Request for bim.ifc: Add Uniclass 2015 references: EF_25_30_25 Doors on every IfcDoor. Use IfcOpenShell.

First a look at what the model holds.

```python
import ifcopenshell

model = ifcopenshell.open("bim.ifc")
print(model.schema)
print("classifications:", [c.Name for c in model.by_type("IfcClassification")])
for ifc_class in ("IfcDoor", "IfcRoof", "IfcStair", "IfcWall", "IfcWindow"):
    print(ifc_class, len(model.by_type(ifc_class)))
```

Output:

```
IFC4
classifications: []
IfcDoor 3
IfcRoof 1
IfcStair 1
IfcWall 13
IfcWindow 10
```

```python
import ifcopenshell
import ifcopenshell.api.classification

model = ifcopenshell.open("bim.ifc")

system = ifcopenshell.api.classification.add_classification(model, classification="Uniclass 2015")

codes = {
    "IfcDoor": ("EF_25_30_25", "Doors"),
}
for ifc_class, (code, name) in codes.items():
    products = model.by_type(ifc_class)
    ifcopenshell.api.classification.add_reference(
        model, products=products, classification=system, identification=code, name=name
    )
    print(code, len(products))

model.write("bim_rev.ifc")
```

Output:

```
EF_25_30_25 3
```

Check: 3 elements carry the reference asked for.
